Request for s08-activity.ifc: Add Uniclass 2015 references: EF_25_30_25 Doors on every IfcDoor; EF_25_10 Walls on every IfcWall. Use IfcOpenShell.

First a look at what the model holds.

```python
import ifcopenshell

model = ifcopenshell.open("s08-activity.ifc")
print(model.schema)
print("classifications:", [c.Name for c in model.by_type("IfcClassification")])
for ifc_class in ("IfcDoor", "IfcRoof", "IfcStair", "IfcWall", "IfcWindow"):
    print(ifc_class, len(model.by_type(ifc_class)))
```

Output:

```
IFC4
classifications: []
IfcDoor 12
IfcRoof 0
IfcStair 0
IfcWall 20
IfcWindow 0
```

```python
import ifcopenshell
import ifcopenshell.api.classification

model = ifcopenshell.open("s08-activity.ifc")

system = ifcopenshell.api.classification.add_classification(model, classification="Uniclass 2015")

codes = {
    "IfcDoor": ("EF_25_30_25", "Doors"),
    "IfcWall": ("EF_25_10", "Walls"),
}
for ifc_class, (code, name) in codes.items():
    products = model.by_type(ifc_class)
    ifcopenshell.api.classification.add_reference(
        model, products=products, classification=system, identification=code, name=name
    )
    print(code, len(products))

model.write("s08-activity-out.ifc")
```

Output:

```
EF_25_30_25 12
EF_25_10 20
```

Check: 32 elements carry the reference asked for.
